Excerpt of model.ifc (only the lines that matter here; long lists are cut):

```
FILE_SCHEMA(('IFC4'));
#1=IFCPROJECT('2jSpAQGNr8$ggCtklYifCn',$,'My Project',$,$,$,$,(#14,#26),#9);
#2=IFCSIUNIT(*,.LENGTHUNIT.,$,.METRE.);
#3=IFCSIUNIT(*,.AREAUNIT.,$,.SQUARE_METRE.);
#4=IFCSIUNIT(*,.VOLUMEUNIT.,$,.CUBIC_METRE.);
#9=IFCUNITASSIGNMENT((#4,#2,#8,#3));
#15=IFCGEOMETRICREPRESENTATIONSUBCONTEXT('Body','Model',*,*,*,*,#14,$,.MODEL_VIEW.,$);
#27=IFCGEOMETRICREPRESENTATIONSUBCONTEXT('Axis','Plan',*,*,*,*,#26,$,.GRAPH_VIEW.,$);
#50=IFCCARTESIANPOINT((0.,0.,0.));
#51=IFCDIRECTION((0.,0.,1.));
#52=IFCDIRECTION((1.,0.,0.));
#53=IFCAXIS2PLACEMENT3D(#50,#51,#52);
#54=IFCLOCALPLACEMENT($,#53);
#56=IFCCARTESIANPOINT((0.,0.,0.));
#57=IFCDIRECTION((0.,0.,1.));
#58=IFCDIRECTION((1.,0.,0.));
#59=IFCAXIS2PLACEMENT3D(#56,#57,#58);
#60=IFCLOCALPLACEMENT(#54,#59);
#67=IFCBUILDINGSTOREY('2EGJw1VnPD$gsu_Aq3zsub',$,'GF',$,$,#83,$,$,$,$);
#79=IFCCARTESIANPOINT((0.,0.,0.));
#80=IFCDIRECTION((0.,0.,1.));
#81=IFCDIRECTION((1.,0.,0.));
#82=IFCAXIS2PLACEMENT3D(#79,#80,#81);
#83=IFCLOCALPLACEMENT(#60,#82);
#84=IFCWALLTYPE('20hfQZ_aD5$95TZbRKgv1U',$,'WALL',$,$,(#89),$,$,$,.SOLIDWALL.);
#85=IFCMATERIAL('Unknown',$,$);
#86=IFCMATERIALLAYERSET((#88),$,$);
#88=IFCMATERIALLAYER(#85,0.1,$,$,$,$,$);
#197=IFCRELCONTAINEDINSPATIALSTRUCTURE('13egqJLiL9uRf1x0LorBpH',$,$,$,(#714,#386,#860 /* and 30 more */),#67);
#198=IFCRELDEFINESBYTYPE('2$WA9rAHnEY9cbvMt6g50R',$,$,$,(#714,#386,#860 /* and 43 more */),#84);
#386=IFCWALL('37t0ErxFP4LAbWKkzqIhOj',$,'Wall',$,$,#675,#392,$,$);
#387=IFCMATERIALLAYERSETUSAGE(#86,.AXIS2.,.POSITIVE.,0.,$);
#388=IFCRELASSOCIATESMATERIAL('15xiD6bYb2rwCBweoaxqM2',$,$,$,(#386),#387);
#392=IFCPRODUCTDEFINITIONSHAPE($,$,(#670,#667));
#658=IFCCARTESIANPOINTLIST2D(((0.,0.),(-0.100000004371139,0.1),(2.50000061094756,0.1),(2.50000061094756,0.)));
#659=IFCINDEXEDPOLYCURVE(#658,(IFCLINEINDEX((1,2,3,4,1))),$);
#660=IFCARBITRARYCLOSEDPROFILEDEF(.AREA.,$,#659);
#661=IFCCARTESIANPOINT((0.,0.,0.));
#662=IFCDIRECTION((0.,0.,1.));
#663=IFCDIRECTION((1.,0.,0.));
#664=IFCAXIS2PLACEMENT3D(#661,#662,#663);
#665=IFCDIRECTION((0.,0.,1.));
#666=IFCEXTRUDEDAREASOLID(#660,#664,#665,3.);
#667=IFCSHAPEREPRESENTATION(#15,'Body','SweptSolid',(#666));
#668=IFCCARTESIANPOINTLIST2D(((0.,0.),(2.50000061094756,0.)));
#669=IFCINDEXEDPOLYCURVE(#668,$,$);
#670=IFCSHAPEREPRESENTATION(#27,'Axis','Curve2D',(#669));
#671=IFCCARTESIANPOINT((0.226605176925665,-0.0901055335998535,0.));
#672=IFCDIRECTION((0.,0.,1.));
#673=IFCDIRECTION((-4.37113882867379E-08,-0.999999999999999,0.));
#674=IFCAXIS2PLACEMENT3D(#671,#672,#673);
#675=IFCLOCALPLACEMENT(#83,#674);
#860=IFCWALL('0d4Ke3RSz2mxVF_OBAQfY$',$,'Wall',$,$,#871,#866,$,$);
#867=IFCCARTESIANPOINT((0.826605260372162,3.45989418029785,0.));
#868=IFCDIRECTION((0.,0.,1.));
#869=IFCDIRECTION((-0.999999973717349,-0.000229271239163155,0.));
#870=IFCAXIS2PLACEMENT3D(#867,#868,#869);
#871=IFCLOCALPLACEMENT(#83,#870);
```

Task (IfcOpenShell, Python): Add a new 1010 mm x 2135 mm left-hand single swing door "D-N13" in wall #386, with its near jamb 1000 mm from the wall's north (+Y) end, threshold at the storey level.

```python
import numpy as np
import ifcopenshell
import ifcopenshell.api.feature
import ifcopenshell.api.geometry
import ifcopenshell.api.root
import ifcopenshell.api.spatial
import ifcopenshell.geom
import ifcopenshell.util.element
import ifcopenshell.util.placement
import ifcopenshell.util.representation
import ifcopenshell.util.shape
import ifcopenshell.util.unit

model = ifcopenshell.open("model.ifc")
unit_scale = ifcopenshell.util.unit.calculate_unit_scale(model)
settings = ifcopenshell.geom.settings()


def volume(element):
    """Net volume in cubic metres, openings subtracted."""
    shape = ifcopenshell.geom.create_shape(settings, element)
    return ifcopenshell.util.shape.get_volume(shape.geometry)


wall = model.by_guid("37t0ErxFP4LAbWKkzqIhOj")
storey = ifcopenshell.util.element.get_container(wall, ifc_class="IfcBuildingStorey")
context = ifcopenshell.util.representation.get_context(model, "Model", "Body", "MODEL_VIEW")
before = volume(wall)

width, height, from_end, sill = 1.01, 2.135, 1, 0.0  # metres

# The wall runs along its own X axis, and the end named is its -X end.
wall_shape = ifcopenshell.geom.create_shape(settings, wall)
x, y, z = ifcopenshell.util.shape.get_vertices(wall_shape.geometry).T
start = x.min() + from_end
face, thickness = float(y.min()), float(y.max() - y.min())
wall_matrix = ifcopenshell.util.placement.get_local_placement(wall.ObjectPlacement)
level = ifcopenshell.util.placement.get_local_placement(storey.ObjectPlacement)[2, 3]


def in_wall(x, y):
    """Placement at x, y metres in the wall's axes, at sill height."""
    matrix = wall_matrix.copy()
    matrix[:, 3] = wall_matrix @ np.array([x / unit_scale, y / unit_scale, 0.0, 1.0])
    matrix[2, 3] = level + sill / unit_scale
    return matrix


# Opening: a box that overshoots both wall faces by 50 mm.
opening = ifcopenshell.api.root.create_entity(model, ifc_class="IfcOpeningElement", predefined_type="OPENING")
box = ifcopenshell.api.geometry.add_wall_representation(
    model, context=context, length=width, height=height, thickness=thickness + 0.1
)
ifcopenshell.api.geometry.assign_representation(model, product=opening, representation=box)
ifcopenshell.api.geometry.edit_object_placement(model, product=opening, matrix=in_wall(start, face - 0.05), is_si=False)
ifcopenshell.api.feature.add_feature(model, feature=opening, element=wall)

door = ifcopenshell.api.root.create_entity(model, ifc_class="IfcDoor", name="D-N13", predefined_type="DOOR")
door.OverallWidth, door.OverallHeight = width / unit_scale, height / unit_scale
door.OperationType = "SINGLE_SWING_LEFT"
body = ifcopenshell.api.geometry.add_door_representation(
    model,
    context=context,
    overall_width=door.OverallWidth,
    overall_height=door.OverallHeight,
    operation_type="SINGLE_SWING_LEFT",
    lining_properties={"LiningDepth": thickness / unit_scale, "ThresholdDepth": thickness / unit_scale},
)
ifcopenshell.api.geometry.assign_representation(model, product=door, representation=body)
ifcopenshell.api.spatial.assign_container(model, products=[door], relating_structure=storey)
ifcopenshell.api.feature.add_filling(model, opening=opening, element=door)

# The lining spans the wall, so the door starts at the wall face.
ifcopenshell.api.geometry.edit_object_placement(model, product=door, matrix=in_wall(start, face), is_si=False)

after = volume(wall)

print(f"wall volume {before:.3f} -> {after:.3f} m3")

model.write("model_updated.ifc")
```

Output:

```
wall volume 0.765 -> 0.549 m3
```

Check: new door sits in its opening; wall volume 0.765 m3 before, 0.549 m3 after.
